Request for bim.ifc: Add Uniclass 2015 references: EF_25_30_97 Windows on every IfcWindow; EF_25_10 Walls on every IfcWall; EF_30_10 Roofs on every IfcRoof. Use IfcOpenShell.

First a look at what the model holds.

```python
import ifcopenshell

model = ifcopenshell.open("bim.ifc")
print(model.schema)
print("classifications:", [c.Name for c in model.by_type("IfcClassification")])
for ifc_class in ("IfcDoor", "IfcRoof", "IfcStair", "IfcWall", "IfcWindow"):
    print(ifc_class, len(model.by_type(ifc_class)))
```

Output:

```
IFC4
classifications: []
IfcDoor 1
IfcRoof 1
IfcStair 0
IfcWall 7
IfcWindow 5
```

```python
import ifcopenshell
import ifcopenshell.api.classification

model = ifcopenshell.open("bim.ifc")

system = ifcopenshell.api.classification.add_classification(model, classification="Uniclass 2015")

codes = {
    "IfcWindow": ("EF_25_30_97", "Windows"),
    "IfcWall": ("EF_25_10", "Walls"),
    "IfcRoof": ("EF_30_10", "Roofs"),
}
for ifc_class, (code, name) in codes.items():
    products = model.by_type(ifc_class)
    ifcopenshell.api.classification.add_reference(
        model, products=products, classification=system, identification=code, name=name
    )
    print(code, len(products))

model.write("bim-out.ifc")
```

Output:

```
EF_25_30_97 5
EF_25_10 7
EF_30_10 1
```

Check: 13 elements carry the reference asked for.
